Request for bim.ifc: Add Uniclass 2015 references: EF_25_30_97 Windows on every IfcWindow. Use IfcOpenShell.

First a look at what the model holds.

```python
import ifcopenshell

model = ifcopenshell.open("bim.ifc")
print(model.schema)
print("classifications:", [c.Name for c in model.by_type("IfcClassification")])
for ifc_class in ("IfcDoor", "IfcRoof", "IfcStair", "IfcWall", "IfcWindow"):
    print(ifc_class, len(model.by_type(ifc_class)))
```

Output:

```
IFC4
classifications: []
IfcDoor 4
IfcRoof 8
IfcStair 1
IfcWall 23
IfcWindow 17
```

```python
import ifcopenshell
import ifcopenshell.api.classification

model = ifcopenshell.open("bim.ifc")

system = ifcopenshell.api.classification.add_classification(model, classification="Uniclass 2015")

codes = {
    "IfcWindow": ("EF_25_30_97", "Windows"),
}
for ifc_class, (code, name) in codes.items():
    products = model.by_type(ifc_class)
    ifcopenshell.api.classification.add_reference(
        model, products=products, classification=system, identification=code, name=name
    )
    print(code, len(products))

model.write("bim_updated.ifc")
```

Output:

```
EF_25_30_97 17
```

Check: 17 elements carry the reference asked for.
